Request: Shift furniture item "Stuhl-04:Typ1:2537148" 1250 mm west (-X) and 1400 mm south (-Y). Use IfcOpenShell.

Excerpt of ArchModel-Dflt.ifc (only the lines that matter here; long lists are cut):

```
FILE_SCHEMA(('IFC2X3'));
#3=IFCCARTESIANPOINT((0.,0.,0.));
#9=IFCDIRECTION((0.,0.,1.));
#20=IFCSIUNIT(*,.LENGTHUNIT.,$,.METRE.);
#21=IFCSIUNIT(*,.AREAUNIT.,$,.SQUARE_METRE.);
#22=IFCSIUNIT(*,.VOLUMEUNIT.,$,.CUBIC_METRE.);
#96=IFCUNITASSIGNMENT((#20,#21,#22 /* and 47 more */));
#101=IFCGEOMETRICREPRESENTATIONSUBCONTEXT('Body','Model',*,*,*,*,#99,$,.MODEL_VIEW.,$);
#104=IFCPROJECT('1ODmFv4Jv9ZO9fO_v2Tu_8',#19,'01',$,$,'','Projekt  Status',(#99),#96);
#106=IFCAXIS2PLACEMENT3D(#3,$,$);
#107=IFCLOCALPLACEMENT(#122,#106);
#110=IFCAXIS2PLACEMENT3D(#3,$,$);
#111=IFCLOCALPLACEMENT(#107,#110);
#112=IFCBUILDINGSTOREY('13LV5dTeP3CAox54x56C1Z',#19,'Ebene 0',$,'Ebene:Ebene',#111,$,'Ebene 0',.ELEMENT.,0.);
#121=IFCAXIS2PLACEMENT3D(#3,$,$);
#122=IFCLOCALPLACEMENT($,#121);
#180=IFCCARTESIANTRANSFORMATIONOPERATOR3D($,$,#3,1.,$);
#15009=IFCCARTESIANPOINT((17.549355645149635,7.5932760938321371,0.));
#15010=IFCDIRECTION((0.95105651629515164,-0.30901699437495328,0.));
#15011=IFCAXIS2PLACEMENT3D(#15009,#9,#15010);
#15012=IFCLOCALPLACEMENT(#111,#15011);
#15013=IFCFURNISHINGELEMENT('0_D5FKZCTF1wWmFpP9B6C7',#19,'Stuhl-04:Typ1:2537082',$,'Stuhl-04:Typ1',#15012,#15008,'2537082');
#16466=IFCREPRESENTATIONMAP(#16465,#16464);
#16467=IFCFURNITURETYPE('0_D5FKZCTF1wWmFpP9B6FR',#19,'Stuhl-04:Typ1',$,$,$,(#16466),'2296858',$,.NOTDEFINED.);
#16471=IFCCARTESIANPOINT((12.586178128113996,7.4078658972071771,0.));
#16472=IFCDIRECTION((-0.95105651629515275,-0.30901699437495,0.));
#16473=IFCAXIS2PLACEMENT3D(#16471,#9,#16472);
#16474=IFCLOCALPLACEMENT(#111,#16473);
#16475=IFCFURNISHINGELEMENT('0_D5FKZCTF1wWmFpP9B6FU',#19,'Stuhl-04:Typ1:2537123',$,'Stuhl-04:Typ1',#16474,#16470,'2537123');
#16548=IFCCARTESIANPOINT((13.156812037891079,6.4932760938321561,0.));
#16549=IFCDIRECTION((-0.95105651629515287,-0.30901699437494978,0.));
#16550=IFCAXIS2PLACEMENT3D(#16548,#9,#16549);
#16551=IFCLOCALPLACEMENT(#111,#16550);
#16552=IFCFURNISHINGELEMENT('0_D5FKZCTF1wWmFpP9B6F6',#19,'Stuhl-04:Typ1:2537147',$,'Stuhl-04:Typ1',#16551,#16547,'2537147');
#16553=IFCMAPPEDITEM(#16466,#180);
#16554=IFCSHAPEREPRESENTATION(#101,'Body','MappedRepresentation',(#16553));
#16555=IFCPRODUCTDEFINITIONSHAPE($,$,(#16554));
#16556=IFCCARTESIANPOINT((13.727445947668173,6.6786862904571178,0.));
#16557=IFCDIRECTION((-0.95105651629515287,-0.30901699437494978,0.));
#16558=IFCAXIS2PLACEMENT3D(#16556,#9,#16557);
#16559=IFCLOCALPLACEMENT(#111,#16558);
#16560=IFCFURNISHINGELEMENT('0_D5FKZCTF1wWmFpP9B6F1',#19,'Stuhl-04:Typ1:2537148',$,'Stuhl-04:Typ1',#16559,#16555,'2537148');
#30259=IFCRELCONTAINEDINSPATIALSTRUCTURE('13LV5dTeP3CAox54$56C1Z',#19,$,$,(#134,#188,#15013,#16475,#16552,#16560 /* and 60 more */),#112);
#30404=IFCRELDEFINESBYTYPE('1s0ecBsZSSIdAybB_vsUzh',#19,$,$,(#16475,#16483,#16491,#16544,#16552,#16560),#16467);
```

```python
import ifcopenshell
import ifcopenshell.api.geometry
import ifcopenshell.util.placement
import ifcopenshell.util.unit

model = ifcopenshell.open("ArchModel-Dflt.ifc")
unit_scale = ifcopenshell.util.unit.calculate_unit_scale(model)

item = model.by_id(16560)
matrix = ifcopenshell.util.placement.get_local_placement(item.ObjectPlacement)
matrix[0, 3] -= 1.25 / unit_scale
matrix[1, 3] -= 1.4 / unit_scale
ifcopenshell.api.geometry.edit_object_placement(model, product=item, matrix=matrix, is_si=False)

print(ifcopenshell.util.placement.get_local_placement(item.ObjectPlacement).round(3) + 0.0)

model.write("ArchModel-Dflt-out.ifc")
```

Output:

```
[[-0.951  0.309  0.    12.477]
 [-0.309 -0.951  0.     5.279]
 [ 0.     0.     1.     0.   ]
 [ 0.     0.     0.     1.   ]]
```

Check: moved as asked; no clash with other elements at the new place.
